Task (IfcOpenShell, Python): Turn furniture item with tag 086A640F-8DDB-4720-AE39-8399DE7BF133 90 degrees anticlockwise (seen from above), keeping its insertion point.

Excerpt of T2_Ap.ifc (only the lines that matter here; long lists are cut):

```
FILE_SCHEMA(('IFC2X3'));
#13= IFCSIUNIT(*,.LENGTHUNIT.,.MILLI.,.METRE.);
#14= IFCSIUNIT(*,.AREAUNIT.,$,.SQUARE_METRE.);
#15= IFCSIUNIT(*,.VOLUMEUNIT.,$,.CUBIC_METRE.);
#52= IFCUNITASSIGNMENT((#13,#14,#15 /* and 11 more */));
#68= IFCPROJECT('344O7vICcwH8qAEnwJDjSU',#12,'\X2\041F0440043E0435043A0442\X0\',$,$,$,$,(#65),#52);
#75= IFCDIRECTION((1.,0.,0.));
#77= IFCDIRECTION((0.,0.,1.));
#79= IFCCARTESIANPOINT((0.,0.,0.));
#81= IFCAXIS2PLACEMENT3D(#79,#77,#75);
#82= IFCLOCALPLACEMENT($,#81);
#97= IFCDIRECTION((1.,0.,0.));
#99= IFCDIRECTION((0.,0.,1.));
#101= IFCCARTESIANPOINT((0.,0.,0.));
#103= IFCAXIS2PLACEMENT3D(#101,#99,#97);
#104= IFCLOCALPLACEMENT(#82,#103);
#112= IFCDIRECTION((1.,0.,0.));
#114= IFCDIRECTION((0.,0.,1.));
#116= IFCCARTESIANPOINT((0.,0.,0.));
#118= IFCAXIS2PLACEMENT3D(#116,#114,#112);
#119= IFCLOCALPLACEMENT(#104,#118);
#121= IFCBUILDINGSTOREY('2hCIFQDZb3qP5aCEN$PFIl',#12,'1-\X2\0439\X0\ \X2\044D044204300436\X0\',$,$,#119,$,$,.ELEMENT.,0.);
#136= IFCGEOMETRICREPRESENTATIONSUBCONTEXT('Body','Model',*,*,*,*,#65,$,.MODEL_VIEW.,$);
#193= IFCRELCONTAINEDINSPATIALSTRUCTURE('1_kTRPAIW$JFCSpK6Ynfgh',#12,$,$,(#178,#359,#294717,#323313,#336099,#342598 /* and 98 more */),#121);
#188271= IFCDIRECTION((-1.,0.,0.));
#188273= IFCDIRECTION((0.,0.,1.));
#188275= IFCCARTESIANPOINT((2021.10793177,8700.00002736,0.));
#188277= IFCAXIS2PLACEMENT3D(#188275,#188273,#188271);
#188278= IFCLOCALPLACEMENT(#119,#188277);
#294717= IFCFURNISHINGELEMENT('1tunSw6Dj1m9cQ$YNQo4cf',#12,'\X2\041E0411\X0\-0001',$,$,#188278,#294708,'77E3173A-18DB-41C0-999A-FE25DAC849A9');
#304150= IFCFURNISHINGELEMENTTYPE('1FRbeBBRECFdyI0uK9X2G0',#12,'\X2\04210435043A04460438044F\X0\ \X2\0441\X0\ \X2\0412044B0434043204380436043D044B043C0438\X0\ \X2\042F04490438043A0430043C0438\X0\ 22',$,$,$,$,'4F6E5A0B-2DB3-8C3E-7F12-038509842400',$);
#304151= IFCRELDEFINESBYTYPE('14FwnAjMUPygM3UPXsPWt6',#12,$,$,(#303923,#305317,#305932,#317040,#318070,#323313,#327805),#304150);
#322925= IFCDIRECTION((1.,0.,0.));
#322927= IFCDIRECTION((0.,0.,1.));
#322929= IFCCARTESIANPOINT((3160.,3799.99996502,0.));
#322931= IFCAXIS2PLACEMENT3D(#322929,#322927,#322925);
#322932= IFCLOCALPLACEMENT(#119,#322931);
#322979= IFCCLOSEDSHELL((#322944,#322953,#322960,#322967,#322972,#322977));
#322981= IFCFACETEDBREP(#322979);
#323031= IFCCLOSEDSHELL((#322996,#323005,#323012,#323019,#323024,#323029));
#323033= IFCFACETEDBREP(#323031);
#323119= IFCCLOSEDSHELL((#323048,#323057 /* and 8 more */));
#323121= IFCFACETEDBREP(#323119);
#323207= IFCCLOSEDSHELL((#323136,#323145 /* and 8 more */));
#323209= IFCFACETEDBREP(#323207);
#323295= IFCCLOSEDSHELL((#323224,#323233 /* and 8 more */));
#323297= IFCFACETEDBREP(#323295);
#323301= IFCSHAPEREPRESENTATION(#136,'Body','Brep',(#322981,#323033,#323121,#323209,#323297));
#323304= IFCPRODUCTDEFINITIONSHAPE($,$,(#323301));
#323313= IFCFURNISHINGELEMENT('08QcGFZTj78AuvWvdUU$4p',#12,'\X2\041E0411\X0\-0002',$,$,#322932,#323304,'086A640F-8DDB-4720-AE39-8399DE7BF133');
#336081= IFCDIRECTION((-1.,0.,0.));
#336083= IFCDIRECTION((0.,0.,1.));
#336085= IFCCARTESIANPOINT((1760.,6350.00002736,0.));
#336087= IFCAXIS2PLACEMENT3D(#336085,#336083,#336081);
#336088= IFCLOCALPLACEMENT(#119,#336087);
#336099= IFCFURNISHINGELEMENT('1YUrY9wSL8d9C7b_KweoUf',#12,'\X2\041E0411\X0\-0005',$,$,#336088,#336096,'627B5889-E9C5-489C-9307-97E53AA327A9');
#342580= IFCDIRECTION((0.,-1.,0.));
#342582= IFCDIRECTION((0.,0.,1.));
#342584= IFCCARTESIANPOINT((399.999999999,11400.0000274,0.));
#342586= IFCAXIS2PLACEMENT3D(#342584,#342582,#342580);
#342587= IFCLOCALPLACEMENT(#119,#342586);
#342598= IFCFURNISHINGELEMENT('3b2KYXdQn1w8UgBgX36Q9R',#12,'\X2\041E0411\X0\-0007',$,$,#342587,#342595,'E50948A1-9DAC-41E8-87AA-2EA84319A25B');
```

```python
import ifcopenshell
import ifcopenshell.api.geometry
import ifcopenshell.util.placement

model = ifcopenshell.open("T2_Ap.ifc")

item = model.by_guid("08QcGFZTj78AuvWvdUU$4p")
matrix = ifcopenshell.util.placement.get_local_placement(item.ObjectPlacement)
matrix = matrix @ ifcopenshell.util.placement.rotation(90, "Z")
ifcopenshell.api.geometry.edit_object_placement(model, product=item, matrix=matrix, is_si=False)

print(ifcopenshell.util.placement.get_local_placement(item.ObjectPlacement).round(3) + 0.0)

model.write("T2_Ap_rev.ifc")
```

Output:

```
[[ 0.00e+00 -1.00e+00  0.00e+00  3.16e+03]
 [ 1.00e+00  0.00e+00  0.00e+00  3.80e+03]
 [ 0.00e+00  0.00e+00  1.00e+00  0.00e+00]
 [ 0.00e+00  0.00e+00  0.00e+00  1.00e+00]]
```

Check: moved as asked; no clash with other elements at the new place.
